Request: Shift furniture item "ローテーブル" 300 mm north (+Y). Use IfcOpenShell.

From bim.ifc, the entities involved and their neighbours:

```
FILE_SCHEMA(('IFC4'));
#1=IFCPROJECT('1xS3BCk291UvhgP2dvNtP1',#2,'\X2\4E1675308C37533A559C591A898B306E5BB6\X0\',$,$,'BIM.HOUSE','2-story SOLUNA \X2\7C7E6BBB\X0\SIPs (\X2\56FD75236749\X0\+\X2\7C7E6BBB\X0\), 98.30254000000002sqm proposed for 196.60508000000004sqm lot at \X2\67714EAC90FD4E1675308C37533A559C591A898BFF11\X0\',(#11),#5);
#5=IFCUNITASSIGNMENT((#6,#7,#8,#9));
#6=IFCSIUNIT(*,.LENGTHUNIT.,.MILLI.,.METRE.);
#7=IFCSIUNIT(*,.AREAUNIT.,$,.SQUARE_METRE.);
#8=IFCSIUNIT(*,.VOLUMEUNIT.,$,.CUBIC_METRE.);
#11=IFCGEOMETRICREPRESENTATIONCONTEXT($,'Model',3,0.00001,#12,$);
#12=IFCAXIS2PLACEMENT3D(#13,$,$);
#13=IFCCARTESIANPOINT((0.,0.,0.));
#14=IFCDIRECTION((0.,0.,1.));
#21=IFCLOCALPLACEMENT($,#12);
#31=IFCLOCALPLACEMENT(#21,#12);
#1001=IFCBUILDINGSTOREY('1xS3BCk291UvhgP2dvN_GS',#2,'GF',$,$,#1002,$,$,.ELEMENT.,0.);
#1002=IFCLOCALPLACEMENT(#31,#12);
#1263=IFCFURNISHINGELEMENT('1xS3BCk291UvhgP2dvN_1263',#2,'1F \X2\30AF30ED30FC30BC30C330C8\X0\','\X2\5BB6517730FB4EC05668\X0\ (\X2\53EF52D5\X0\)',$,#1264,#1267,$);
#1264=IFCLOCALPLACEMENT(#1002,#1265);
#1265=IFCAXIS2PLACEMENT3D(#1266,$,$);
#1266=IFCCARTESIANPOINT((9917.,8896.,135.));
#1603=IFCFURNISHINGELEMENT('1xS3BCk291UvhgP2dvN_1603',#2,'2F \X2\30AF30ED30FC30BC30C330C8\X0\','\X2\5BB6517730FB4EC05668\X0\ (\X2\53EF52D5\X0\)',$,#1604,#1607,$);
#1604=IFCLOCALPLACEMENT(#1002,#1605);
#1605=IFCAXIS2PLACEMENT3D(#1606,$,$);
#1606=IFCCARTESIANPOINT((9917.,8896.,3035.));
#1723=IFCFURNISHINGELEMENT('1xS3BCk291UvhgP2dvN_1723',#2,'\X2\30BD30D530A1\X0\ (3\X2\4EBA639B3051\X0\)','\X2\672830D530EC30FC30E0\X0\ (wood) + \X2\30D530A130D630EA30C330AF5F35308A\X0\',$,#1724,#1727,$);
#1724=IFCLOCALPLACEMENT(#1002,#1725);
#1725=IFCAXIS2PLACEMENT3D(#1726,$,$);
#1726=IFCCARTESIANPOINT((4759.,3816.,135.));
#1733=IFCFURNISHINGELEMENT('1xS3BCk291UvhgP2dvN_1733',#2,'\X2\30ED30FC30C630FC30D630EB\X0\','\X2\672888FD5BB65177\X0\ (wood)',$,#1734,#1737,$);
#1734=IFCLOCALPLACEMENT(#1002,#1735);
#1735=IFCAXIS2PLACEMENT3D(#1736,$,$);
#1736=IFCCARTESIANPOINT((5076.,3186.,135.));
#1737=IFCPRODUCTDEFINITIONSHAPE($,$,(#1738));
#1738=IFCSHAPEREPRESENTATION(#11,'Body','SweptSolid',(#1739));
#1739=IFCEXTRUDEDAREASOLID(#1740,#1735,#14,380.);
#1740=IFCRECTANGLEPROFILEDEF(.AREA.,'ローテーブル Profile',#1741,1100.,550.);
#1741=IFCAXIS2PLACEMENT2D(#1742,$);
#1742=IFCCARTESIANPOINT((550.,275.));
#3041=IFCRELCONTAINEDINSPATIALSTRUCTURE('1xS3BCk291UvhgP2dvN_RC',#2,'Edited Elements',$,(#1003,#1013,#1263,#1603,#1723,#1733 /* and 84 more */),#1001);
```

```python
import ifcopenshell
import ifcopenshell.api.geometry
import ifcopenshell.util.placement

model = ifcopenshell.open("bim.ifc")

item = model.by_guid("1xS3BCk291UvhgP2dvN_1733")
matrix = ifcopenshell.util.placement.get_local_placement(item.ObjectPlacement)
matrix[1, 3] += 300.0
ifcopenshell.api.geometry.edit_object_placement(model, product=item, matrix=matrix, is_si=False)

print(ifcopenshell.util.placement.get_local_placement(item.ObjectPlacement).round(3) + 0.0)

model.write("bim_rev.ifc")
```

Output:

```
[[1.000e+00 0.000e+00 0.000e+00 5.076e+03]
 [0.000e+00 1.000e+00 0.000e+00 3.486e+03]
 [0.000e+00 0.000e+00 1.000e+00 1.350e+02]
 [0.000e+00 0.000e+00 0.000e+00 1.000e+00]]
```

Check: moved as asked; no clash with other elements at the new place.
